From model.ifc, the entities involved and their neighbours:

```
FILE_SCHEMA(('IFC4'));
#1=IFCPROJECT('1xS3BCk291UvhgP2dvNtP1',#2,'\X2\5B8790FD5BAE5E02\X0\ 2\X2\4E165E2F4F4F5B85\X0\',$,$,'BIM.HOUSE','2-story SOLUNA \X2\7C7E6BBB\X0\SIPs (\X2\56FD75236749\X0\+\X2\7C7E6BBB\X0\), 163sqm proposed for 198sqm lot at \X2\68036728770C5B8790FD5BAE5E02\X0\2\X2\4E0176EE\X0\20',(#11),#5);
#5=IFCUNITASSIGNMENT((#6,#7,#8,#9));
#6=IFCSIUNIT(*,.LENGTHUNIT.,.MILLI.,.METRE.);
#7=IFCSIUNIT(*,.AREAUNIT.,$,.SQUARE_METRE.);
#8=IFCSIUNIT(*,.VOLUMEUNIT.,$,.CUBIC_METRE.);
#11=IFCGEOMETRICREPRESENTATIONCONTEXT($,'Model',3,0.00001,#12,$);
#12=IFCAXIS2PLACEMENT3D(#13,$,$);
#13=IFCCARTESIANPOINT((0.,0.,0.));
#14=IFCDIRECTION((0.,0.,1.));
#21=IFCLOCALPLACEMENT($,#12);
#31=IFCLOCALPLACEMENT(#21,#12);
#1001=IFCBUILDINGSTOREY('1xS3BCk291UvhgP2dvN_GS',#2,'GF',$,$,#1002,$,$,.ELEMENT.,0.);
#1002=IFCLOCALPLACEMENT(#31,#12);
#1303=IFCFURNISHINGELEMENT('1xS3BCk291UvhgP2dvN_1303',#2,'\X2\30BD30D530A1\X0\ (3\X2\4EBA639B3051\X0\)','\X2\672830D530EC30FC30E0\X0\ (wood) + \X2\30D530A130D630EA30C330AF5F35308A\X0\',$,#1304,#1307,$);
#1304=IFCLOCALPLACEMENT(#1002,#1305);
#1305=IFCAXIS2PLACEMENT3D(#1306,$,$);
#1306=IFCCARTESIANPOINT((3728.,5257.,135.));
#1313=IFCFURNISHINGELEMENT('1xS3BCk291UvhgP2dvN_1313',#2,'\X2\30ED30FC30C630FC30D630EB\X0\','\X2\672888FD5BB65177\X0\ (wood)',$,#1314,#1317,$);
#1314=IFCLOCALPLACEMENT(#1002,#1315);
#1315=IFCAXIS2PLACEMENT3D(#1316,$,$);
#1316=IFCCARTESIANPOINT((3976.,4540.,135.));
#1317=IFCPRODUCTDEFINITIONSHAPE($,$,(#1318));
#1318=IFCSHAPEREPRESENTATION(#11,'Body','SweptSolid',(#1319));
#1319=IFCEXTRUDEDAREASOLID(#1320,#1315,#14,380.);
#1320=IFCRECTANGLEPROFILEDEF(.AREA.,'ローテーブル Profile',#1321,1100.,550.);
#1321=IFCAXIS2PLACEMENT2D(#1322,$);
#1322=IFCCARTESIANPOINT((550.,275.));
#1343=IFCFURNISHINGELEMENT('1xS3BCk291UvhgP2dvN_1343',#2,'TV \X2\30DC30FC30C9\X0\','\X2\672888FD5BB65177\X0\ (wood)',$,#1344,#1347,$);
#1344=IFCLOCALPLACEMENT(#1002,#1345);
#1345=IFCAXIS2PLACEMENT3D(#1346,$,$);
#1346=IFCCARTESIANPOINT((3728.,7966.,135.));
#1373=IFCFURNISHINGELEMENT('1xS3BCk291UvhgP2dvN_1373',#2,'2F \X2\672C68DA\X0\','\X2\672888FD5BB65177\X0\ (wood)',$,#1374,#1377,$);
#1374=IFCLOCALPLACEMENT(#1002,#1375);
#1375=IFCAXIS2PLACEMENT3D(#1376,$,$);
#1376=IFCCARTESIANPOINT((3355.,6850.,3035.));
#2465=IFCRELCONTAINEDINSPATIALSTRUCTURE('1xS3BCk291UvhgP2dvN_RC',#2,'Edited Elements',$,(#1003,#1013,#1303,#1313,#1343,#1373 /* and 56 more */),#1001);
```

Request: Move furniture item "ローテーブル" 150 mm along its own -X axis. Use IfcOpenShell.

```python
import ifcopenshell
import ifcopenshell.api.geometry
import ifcopenshell.util.placement

model = ifcopenshell.open("model.ifc")

item = model.by_guid("1xS3BCk291UvhgP2dvN_1313")
matrix = ifcopenshell.util.placement.get_local_placement(item.ObjectPlacement)
matrix[:3, 3] -= matrix[:3, 0] * 150.0
ifcopenshell.api.geometry.edit_object_placement(model, product=item, matrix=matrix, is_si=False)

print(ifcopenshell.util.placement.get_local_placement(item.ObjectPlacement).round(3) + 0.0)

model.write("model_v2.ifc")
```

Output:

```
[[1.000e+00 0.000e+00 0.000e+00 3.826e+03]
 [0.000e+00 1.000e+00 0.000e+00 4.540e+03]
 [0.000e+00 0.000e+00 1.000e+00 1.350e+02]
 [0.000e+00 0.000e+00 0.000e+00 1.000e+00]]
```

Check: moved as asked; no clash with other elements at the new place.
